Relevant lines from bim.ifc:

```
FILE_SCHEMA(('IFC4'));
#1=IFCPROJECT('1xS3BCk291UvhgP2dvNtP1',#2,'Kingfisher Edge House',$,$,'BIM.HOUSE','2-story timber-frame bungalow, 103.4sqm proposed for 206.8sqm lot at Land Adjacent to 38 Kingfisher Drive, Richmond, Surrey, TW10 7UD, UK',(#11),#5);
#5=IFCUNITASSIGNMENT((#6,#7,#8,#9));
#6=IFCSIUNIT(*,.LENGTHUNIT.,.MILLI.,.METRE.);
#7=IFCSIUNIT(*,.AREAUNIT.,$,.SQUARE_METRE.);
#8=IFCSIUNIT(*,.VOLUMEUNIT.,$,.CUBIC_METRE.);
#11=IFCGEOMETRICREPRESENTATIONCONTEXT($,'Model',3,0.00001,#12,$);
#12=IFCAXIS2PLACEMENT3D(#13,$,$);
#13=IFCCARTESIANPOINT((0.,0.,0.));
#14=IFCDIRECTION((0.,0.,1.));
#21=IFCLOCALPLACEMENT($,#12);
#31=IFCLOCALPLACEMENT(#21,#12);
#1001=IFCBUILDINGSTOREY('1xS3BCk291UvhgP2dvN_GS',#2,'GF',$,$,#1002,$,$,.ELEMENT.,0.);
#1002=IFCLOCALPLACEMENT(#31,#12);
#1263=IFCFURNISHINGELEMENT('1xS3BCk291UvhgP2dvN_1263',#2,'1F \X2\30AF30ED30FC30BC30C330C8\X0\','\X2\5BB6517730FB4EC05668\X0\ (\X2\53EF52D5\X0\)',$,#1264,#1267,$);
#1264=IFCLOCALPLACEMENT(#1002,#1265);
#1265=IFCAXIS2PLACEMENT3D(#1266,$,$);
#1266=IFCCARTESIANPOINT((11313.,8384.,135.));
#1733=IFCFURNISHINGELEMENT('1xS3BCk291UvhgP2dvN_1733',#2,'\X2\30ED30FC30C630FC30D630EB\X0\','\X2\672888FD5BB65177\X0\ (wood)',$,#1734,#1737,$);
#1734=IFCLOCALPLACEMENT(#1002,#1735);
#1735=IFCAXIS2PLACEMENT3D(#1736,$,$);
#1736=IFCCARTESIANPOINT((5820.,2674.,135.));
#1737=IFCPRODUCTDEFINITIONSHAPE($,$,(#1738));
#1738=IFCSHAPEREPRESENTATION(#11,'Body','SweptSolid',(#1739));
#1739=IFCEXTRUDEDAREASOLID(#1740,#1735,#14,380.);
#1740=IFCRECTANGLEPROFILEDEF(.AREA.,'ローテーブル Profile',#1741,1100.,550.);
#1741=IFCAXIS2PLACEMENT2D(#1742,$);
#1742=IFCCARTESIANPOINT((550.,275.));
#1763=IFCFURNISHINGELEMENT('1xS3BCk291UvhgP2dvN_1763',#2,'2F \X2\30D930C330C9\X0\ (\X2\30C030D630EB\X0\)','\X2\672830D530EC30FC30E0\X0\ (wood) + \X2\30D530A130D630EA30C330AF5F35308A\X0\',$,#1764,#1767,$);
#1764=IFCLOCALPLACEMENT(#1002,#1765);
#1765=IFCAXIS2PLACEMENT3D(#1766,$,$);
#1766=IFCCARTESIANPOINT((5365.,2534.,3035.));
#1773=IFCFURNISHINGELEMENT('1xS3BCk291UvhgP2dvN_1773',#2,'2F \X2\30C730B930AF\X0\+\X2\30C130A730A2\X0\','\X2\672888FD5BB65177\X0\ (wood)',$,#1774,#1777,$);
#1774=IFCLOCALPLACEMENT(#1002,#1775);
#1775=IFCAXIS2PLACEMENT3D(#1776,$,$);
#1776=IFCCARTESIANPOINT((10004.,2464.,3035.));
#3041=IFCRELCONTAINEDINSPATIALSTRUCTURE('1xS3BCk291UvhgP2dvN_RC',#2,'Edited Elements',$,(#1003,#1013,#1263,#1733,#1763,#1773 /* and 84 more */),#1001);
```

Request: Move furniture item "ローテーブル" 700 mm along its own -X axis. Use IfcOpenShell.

```python
import ifcopenshell
import ifcopenshell.api.geometry
import ifcopenshell.util.placement

model = ifcopenshell.open("bim.ifc")

item = model.by_id(1733)
matrix = ifcopenshell.util.placement.get_local_placement(item.ObjectPlacement)
matrix[:3, 3] -= matrix[:3, 0] * 700.0
ifcopenshell.api.geometry.edit_object_placement(model, product=item, matrix=matrix, is_si=False)

print(ifcopenshell.util.placement.get_local_placement(item.ObjectPlacement).round(3) + 0.0)

model.write("bim_updated.ifc")
```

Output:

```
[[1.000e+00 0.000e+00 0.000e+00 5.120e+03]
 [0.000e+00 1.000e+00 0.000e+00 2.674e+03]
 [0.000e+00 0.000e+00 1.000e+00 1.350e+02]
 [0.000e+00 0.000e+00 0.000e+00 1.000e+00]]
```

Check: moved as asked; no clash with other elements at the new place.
